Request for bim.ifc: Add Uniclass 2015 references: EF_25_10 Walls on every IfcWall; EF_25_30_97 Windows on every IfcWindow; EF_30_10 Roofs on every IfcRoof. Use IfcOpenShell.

First a look at what the model holds.

```python
import ifcopenshell

model = ifcopenshell.open("bim.ifc")
print(model.schema)
print("classifications:", [c.Name for c in model.by_type("IfcClassification")])
for ifc_class in ("IfcDoor", "IfcRoof", "IfcStair", "IfcWall", "IfcWindow"):
    print(ifc_class, len(model.by_type(ifc_class)))
```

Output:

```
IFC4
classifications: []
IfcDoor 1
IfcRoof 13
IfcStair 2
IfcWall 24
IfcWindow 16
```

```python
import ifcopenshell
import ifcopenshell.api.classification

model = ifcopenshell.open("bim.ifc")

system = ifcopenshell.api.classification.add_classification(model, classification="Uniclass 2015")

codes = {
    "IfcWall": ("EF_25_10", "Walls"),
    "IfcWindow": ("EF_25_30_97", "Windows"),
    "IfcRoof": ("EF_30_10", "Roofs"),
}
for ifc_class, (code, name) in codes.items():
    products = model.by_type(ifc_class)
    ifcopenshell.api.classification.add_reference(
        model, products=products, classification=system, identification=code, name=name
    )
    print(code, len(products))

model.write("bim_v2.ifc")
```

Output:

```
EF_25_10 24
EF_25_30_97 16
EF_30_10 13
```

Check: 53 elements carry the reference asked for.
